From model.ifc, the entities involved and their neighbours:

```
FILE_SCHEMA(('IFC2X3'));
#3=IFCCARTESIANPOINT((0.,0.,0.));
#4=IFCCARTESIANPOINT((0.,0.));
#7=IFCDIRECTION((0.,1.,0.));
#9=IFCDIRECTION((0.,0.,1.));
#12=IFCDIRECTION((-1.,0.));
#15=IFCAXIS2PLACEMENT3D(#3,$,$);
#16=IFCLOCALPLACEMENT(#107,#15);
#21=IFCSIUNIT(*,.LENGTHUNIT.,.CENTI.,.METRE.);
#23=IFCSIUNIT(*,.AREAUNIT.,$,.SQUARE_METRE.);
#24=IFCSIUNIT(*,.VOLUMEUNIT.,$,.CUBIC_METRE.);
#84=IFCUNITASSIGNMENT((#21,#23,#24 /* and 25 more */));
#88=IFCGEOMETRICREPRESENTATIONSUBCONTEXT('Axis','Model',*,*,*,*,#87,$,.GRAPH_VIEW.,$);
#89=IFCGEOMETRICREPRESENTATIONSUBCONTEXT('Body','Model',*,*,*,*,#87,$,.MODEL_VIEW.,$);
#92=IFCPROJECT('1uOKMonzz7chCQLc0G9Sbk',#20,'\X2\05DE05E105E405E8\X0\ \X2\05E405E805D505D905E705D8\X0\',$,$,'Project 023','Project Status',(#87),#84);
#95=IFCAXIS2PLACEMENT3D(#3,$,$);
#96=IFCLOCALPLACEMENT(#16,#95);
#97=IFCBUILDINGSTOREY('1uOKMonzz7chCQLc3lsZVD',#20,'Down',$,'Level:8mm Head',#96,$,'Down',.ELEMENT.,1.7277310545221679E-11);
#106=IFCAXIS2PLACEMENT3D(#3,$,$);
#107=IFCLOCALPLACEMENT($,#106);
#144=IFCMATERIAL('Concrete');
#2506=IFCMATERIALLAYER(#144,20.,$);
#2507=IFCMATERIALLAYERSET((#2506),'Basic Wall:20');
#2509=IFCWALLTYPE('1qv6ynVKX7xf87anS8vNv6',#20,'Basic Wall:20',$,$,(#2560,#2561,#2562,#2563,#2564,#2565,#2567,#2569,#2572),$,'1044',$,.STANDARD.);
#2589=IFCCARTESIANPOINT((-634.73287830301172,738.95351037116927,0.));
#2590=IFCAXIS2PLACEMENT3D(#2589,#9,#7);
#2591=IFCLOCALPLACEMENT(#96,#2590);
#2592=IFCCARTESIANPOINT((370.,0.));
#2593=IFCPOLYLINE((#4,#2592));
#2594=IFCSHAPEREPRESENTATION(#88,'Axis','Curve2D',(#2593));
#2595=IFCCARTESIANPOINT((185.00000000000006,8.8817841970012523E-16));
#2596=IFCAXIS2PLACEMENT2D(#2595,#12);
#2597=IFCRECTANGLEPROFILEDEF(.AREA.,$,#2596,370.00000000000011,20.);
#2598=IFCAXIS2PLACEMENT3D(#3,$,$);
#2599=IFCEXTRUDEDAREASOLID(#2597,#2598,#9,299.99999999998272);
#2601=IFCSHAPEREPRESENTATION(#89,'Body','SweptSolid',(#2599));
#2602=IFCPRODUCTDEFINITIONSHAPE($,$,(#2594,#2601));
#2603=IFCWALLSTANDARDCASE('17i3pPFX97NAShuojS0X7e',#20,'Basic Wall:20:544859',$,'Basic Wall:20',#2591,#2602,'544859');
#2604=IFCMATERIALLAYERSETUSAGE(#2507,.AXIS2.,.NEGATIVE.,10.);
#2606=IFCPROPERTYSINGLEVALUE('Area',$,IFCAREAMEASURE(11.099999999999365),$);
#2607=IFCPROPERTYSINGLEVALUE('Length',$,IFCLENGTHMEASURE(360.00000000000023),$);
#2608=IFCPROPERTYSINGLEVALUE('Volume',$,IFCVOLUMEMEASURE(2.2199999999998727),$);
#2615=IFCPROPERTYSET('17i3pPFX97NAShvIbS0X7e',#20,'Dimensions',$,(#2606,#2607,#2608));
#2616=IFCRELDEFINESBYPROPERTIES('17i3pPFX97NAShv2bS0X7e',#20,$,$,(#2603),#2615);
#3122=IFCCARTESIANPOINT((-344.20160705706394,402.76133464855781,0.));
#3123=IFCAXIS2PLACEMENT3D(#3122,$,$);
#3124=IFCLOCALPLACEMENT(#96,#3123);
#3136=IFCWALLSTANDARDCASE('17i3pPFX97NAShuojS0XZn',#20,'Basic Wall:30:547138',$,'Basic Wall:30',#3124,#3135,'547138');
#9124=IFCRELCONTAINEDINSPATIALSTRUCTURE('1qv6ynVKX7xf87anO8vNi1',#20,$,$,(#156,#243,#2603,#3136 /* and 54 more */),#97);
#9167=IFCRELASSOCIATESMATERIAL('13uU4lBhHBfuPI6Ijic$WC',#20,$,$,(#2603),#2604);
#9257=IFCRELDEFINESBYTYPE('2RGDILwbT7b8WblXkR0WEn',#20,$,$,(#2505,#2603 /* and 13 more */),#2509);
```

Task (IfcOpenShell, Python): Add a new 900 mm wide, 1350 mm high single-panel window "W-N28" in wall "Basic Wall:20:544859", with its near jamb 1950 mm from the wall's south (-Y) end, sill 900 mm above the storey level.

```python
import numpy as np
import ifcopenshell
import ifcopenshell.api.feature
import ifcopenshell.api.geometry
import ifcopenshell.api.pset
import ifcopenshell.api.root
import ifcopenshell.api.spatial
import ifcopenshell.api.type
import ifcopenshell.geom
import ifcopenshell.util.element
import ifcopenshell.util.placement
import ifcopenshell.util.representation
import ifcopenshell.util.shape
import ifcopenshell.util.unit

model = ifcopenshell.open("model.ifc")
unit_scale = ifcopenshell.util.unit.calculate_unit_scale(model)
area_scale = ifcopenshell.util.unit.calculate_unit_scale(model, "AREAUNIT")
volume_scale = ifcopenshell.util.unit.calculate_unit_scale(model, "VOLUMEUNIT")
settings = ifcopenshell.geom.settings()


def volume(element):
    """Net volume in cubic metres, openings subtracted."""
    shape = ifcopenshell.geom.create_shape(settings, element)
    return ifcopenshell.util.shape.get_volume(shape.geometry)


wall = model.by_guid("17i3pPFX97NAShuojS0X7e")
storey = ifcopenshell.util.element.get_container(wall, ifc_class="IfcBuildingStorey")
context = ifcopenshell.util.representation.get_context(model, "Model", "Body", "MODEL_VIEW")
before = volume(wall)

width, height, from_end, sill = 0.9, 1.35, 1.95, 0.9  # metres

# The wall runs along its own X axis, and the end named is its -X end.
wall_shape = ifcopenshell.geom.create_shape(settings, wall)
x, y, z = ifcopenshell.util.shape.get_vertices(wall_shape.geometry).T
start = x.min() + from_end
face, thickness = float(y.min()), float(y.max() - y.min())
wall_matrix = ifcopenshell.util.placement.get_local_placement(wall.ObjectPlacement)
level = ifcopenshell.util.placement.get_local_placement(storey.ObjectPlacement)[2, 3]


def in_wall(x, y):
    """Placement at x, y metres in the wall's axes, at sill height."""
    matrix = wall_matrix.copy()
    matrix[:, 3] = wall_matrix @ np.array([x / unit_scale, y / unit_scale, 0.0, 1.0])
    matrix[2, 3] = level + sill / unit_scale
    return matrix


# Opening: a box that overshoots both wall faces by 50 mm.
opening = ifcopenshell.api.root.create_entity(model, ifc_class="IfcOpeningElement")
box = ifcopenshell.api.geometry.add_wall_representation(
    model, context=context, length=width, height=height, thickness=thickness + 0.1
)
ifcopenshell.api.geometry.assign_representation(model, product=opening, representation=box)
ifcopenshell.api.geometry.edit_object_placement(model, product=opening, matrix=in_wall(start, face - 0.05), is_si=False)
ifcopenshell.api.feature.add_feature(model, feature=opening, element=wall)

window = ifcopenshell.api.root.create_entity(model, ifc_class="IfcWindow", name="W-N28")
window.OverallWidth, window.OverallHeight = width / unit_scale, height / unit_scale
body = ifcopenshell.api.geometry.add_window_representation(
    model,
    context=context,
    overall_width=window.OverallWidth,
    overall_height=window.OverallHeight,
    partition_type="SINGLE_PANEL",
)
ifcopenshell.api.geometry.assign_representation(model, product=window, representation=body)
ifcopenshell.api.spatial.assign_container(model, products=[window], relating_structure=storey)
fills = ifcopenshell.api.feature.add_filling(model, opening=opening, element=window)
fills.OwnerHistory = window.OwnerHistory  # required in IFC2X3

# IFC2X3 keeps the operation on the window style.
style = ifcopenshell.api.root.create_entity(model, ifc_class="IfcWindowStyle", name="W-N28")
style.OperationType, style.ConstructionType = "SINGLE_PANEL", "NOTDEFINED"
style.ParameterTakesPrecedence = style.Sizeable = False
ifcopenshell.api.type.assign_type(model, related_objects=[window], relating_type=style)

# Centre the window in the wall's thickness.
ifcopenshell.api.geometry.edit_object_placement(model, product=window, matrix=in_wall(start, face), is_si=False)
window_shape = ifcopenshell.geom.create_shape(settings, window)
depth = ifcopenshell.util.shape.get_vertices(window_shape.geometry)[:, 1]
offset = face + thickness / 2 - (depth.min() + depth.max()) / 2
ifcopenshell.api.geometry.edit_object_placement(model, product=window, matrix=in_wall(start, offset), is_si=False)

after = volume(wall)

# Update the wall's stored quantities.
pset = model.by_id(ifcopenshell.util.element.get_pset(wall, "Dimensions", should_inherit=False)["id"])
ifcopenshell.api.pset.edit_pset(model, pset=pset, properties={
    "Area": model.create_entity("IfcAreaMeasure", after / thickness / area_scale),
    "Volume": model.create_entity("IfcVolumeMeasure", after / volume_scale),
})

print(f"wall volume {before:.3f} -> {after:.3f} m3")

model.write("model_rev.ifc")
```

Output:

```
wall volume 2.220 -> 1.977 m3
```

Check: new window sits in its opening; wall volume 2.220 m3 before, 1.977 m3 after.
